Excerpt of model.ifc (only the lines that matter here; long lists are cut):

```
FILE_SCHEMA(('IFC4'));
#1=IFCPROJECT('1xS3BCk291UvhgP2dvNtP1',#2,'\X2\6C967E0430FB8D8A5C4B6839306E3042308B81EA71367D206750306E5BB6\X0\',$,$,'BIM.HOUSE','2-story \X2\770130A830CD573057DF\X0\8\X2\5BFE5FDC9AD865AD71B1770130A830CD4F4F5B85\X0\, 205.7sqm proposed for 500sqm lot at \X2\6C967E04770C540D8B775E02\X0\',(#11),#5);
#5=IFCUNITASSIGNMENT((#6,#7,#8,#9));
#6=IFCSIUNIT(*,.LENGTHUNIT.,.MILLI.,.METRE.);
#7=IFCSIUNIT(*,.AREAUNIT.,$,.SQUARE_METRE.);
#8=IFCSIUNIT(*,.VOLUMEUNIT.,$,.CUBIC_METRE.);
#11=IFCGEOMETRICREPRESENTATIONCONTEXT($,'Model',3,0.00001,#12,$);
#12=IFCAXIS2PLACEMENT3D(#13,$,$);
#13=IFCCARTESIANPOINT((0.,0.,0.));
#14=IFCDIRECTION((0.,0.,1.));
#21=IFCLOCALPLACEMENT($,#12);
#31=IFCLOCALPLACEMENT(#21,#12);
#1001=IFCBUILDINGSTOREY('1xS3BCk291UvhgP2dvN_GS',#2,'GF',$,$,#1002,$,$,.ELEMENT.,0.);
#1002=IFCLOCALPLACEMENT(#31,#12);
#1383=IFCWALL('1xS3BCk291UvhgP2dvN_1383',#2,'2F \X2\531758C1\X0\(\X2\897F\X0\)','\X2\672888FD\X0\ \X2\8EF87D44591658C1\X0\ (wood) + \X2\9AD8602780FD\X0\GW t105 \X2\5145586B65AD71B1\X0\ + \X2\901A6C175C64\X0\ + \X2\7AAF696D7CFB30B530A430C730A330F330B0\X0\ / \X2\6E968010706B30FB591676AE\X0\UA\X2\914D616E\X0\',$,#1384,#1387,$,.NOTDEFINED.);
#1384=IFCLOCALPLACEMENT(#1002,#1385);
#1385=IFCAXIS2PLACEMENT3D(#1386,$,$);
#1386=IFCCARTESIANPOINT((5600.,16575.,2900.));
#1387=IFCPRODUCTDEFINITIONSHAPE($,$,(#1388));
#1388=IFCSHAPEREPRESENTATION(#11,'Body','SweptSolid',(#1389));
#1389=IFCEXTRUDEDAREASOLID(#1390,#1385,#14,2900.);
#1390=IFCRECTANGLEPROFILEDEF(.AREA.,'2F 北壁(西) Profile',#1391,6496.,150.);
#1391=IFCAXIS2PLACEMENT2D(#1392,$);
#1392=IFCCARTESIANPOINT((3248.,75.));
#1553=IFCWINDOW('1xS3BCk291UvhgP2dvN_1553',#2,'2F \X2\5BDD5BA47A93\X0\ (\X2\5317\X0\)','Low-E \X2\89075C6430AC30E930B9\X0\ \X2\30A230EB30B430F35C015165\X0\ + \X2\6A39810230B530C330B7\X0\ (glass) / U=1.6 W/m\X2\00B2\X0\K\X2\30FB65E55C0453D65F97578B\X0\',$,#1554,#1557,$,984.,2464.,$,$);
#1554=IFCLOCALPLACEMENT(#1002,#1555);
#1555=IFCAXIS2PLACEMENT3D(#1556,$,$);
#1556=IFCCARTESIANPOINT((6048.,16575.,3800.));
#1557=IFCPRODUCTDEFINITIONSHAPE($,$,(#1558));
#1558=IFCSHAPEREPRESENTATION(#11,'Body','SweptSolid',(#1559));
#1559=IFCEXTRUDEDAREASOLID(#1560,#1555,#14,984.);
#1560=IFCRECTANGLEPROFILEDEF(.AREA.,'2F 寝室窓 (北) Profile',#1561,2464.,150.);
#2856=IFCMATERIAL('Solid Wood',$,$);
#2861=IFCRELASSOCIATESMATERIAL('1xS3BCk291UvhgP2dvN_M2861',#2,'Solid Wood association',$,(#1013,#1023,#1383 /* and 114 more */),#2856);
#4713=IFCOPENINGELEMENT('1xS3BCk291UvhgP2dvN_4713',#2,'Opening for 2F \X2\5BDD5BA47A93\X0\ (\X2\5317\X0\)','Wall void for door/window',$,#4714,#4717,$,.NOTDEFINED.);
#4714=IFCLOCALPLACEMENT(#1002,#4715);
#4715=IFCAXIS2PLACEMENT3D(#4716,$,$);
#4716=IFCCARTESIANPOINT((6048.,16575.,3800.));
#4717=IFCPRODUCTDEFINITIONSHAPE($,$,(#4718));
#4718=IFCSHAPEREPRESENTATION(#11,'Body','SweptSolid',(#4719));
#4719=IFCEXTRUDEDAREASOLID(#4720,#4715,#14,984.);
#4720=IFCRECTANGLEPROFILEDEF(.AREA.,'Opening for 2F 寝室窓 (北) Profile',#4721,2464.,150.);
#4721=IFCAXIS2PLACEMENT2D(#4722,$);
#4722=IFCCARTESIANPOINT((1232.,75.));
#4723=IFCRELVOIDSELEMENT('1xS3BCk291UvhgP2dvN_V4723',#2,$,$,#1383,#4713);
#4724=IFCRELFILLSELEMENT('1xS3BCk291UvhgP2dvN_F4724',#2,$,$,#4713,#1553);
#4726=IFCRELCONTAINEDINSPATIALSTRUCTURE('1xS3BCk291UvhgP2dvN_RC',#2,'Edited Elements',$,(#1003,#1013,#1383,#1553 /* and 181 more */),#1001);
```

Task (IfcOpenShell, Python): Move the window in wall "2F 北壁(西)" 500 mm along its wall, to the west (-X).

```python
import ifcopenshell
import ifcopenshell.api.geometry
import ifcopenshell.util.placement

model = ifcopenshell.open("model.ifc")

window = model.by_id(1553)
opening = window.FillsVoids[0].RelatingOpeningElement
wall = opening.VoidsElements[0].RelatingBuildingElement

wall_matrix = ifcopenshell.util.placement.get_local_placement(wall.ObjectPlacement)
shift = wall_matrix[:3, 0] * -500.0
before = ifcopenshell.util.placement.get_local_placement(window.ObjectPlacement)[:3, 3].copy()

# The window is not placed relative to its opening, so move both.
for product in (opening, window):
    matrix = ifcopenshell.util.placement.get_local_placement(product.ObjectPlacement)
    matrix[:3, 3] += shift
    ifcopenshell.api.geometry.edit_object_placement(model, product=product, matrix=matrix, is_si=False)

after = ifcopenshell.util.placement.get_local_placement(window.ObjectPlacement)[:3, 3]
print("window moved by", (after - before).round(3) + 0.0)

model.write("model_updated.ifc")
```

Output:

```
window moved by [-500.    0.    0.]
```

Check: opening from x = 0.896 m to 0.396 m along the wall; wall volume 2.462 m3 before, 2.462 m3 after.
